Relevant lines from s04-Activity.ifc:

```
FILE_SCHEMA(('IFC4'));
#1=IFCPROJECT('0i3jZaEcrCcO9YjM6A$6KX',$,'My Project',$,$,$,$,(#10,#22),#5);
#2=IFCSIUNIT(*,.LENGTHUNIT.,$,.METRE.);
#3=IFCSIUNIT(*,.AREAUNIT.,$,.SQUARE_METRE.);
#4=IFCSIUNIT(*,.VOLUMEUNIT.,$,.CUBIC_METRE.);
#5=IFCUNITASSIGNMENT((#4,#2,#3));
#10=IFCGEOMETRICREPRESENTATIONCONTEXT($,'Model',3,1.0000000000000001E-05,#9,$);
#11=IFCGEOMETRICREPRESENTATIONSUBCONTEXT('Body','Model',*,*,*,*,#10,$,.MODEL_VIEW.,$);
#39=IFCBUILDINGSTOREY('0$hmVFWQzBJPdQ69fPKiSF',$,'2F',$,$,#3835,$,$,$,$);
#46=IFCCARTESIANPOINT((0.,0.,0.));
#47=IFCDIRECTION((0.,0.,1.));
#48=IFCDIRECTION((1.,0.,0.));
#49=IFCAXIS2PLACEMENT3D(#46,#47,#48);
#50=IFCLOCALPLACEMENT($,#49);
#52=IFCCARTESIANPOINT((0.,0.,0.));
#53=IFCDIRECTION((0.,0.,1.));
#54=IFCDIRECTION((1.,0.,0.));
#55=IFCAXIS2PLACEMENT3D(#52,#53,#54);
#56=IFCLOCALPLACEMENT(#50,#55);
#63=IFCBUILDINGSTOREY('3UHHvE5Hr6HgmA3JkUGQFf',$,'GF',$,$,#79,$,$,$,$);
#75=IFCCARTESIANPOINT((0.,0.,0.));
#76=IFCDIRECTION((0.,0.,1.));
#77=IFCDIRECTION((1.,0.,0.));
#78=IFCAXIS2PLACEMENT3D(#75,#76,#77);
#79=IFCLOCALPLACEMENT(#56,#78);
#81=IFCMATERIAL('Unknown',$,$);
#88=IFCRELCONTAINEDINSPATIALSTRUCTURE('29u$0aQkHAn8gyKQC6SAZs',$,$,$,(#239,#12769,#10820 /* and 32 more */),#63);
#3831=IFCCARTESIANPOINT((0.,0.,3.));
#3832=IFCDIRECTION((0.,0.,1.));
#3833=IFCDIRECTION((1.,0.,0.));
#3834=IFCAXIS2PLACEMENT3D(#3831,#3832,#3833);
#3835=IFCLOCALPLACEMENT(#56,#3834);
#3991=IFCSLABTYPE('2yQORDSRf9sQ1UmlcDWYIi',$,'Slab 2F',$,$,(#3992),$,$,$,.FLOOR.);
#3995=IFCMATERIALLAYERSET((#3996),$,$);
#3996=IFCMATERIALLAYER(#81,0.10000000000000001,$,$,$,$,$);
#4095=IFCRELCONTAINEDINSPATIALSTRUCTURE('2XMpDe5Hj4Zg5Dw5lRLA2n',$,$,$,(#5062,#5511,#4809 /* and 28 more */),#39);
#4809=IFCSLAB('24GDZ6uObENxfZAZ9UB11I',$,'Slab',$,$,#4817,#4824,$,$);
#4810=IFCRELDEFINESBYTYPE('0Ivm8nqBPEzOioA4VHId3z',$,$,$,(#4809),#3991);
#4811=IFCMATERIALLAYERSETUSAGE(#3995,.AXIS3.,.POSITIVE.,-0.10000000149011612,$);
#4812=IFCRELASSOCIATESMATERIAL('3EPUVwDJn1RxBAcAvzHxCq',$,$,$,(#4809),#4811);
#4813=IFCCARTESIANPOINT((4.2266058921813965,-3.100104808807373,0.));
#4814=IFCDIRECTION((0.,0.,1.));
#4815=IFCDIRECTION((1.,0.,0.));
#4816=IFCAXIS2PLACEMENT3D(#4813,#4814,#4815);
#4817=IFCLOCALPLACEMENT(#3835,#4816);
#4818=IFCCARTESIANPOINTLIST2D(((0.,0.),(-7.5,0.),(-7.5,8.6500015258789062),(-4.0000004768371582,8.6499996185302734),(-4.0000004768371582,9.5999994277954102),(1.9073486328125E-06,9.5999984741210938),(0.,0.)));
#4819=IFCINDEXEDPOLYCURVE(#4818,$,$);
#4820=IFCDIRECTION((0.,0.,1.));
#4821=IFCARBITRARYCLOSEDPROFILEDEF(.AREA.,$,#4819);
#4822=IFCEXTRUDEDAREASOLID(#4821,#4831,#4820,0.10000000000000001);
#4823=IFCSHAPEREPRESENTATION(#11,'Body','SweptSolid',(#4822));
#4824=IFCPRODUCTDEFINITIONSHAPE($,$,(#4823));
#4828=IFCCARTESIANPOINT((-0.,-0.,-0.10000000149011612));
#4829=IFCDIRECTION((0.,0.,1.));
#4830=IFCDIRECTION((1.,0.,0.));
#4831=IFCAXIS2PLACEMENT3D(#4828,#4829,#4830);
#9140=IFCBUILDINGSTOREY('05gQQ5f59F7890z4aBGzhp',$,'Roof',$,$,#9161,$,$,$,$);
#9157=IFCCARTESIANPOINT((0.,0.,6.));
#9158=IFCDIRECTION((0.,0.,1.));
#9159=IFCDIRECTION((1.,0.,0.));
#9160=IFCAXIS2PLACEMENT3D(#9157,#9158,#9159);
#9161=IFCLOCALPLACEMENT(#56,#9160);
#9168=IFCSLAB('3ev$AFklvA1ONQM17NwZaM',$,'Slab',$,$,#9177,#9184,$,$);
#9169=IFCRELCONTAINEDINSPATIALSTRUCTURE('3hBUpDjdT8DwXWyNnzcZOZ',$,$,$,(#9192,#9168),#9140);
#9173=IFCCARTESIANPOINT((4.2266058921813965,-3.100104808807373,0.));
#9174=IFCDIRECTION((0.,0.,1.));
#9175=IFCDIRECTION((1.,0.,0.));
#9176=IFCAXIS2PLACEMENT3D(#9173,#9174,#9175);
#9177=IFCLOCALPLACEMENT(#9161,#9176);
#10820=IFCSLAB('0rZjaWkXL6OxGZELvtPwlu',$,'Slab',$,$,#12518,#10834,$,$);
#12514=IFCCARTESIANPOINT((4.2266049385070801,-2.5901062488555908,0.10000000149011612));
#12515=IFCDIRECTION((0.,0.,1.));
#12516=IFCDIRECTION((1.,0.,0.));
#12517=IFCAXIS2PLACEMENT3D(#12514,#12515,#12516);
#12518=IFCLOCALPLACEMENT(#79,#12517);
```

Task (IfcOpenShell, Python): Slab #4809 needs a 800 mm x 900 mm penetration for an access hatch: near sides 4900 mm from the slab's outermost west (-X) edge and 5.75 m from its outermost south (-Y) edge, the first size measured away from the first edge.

```python
import numpy as np
import ifcopenshell
import ifcopenshell.api.feature
import ifcopenshell.api.geometry
import ifcopenshell.api.root
import ifcopenshell.geom
import ifcopenshell.util.placement
import ifcopenshell.util.representation
import ifcopenshell.util.shape
import ifcopenshell.util.unit

model = ifcopenshell.open("s04-Activity.ifc")
unit_scale = ifcopenshell.util.unit.calculate_unit_scale(model)
settings = ifcopenshell.geom.settings()


def volume(element):
    """Net volume in cubic metres, openings subtracted."""
    shape = ifcopenshell.geom.create_shape(settings, element)
    return ifcopenshell.util.shape.get_volume(shape.geometry)


slab = model.by_guid("24GDZ6uObENxfZAZ9UB11I")
before = volume(slab)

# Extent in the slab's own axes, in metres. The edges named are its -X and -Y sides.
slab_shape = ifcopenshell.geom.create_shape(settings, slab)
vertices = ifcopenshell.util.shape.get_vertices(slab_shape.geometry)
x_min, y_min, bottom = vertices.min(axis=0)
top = vertices[:, 2].max()

opening = ifcopenshell.api.root.create_entity(model, ifc_class="IfcOpeningElement", name="Access hatch opening", predefined_type="OPENING")
context = ifcopenshell.util.representation.get_context(model, "Model", "Body", "MODEL_VIEW")
width, depth = 0.8, 0.9
outline = [(0.0, 0.0), (width, 0.0), (width, depth), (0.0, depth), (0.0, 0.0)]
# Overshoot both faces by 50 mm so the cut is clean.
shape = ifcopenshell.api.geometry.add_slab_representation(
    model, context=context, depth=top - bottom + 0.1, polyline=outline
)
ifcopenshell.api.geometry.assign_representation(model, product=opening, representation=shape)

matrix = ifcopenshell.util.placement.get_local_placement(slab.ObjectPlacement)
matrix[:, 3] = matrix @ np.append(np.array([x_min + 4.9, y_min + 5.75, bottom - 0.05]) / unit_scale, 1.0)
ifcopenshell.api.geometry.edit_object_placement(model, product=opening, matrix=matrix, is_si=False)
ifcopenshell.api.feature.add_feature(model, feature=opening, element=slab)

after = volume(slab)

print(f"slab volume {before:.3f} -> {after:.3f} m3")

model.write("s04-Activity-out.ifc")
```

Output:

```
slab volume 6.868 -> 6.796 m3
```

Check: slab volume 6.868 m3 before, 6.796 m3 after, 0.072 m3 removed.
